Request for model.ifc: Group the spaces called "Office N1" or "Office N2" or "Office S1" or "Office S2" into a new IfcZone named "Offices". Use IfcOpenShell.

First a look at what the model holds.

```python
import ifcopenshell

model = ifcopenshell.open("model.ifc")
print(model.schema)
seen = {}
for space in model.by_type("IfcSpace"):
    seen[space.LongName] = seen.get(space.LongName, 0) + 1
for name, count in sorted(seen.items(), key=str):
    print(count, "x", name)
print("zones:", [z.Name for z in model.by_type("IfcZone")][:20])
```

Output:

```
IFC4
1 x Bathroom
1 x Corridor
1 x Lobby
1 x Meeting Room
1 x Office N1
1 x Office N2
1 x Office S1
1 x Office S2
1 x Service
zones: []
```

```python
import ifcopenshell
import ifcopenshell.api.group
import ifcopenshell.api.root

model = ifcopenshell.open("model.ifc")

names = {"Office N1", "Office N2", "Office S1", "Office S2"}
spaces = [s for s in model.by_type("IfcSpace") if s.LongName in names]

zone = ifcopenshell.api.root.create_entity(model, ifc_class="IfcZone", name="Offices")
ifcopenshell.api.group.assign_group(model, products=spaces, group=zone)
print(len(spaces), "spaces in", zone.Name)

model.write("model-out.ifc")
```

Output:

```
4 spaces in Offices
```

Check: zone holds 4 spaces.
